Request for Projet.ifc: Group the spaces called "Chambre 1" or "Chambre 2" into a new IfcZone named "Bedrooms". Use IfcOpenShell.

First a look at what the model holds.

```python
import ifcopenshell

model = ifcopenshell.open("Projet.ifc")
print(model.schema)
seen = {}
for space in model.by_type("IfcSpace"):
    seen[space.LongName] = seen.get(space.LongName, 0) + 1
for name, count in sorted(seen.items(), key=str):
    print(count, "x", name)
print("zones:", [z.Name for z in model.by_type("IfcZone")][:20])
```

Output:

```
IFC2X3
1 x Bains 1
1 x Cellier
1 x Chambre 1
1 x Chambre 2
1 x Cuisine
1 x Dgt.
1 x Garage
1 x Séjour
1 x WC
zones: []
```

```python
import ifcopenshell
import ifcopenshell.api.group
import ifcopenshell.api.root

model = ifcopenshell.open("Projet.ifc")

names = {"Chambre 1", "Chambre 2"}
spaces = [s for s in model.by_type("IfcSpace") if s.LongName in names]

zone = ifcopenshell.api.root.create_entity(model, ifc_class="IfcZone", name="Bedrooms")
ifcopenshell.api.group.assign_group(model, products=spaces, group=zone)
print(len(spaces), "spaces in", zone.Name)

model.write("Projet_rev.ifc")
```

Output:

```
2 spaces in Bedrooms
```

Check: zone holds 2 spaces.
